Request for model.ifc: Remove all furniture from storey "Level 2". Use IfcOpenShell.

First a look at what the model holds.

```python
import ifcopenshell
import ifcopenshell.util.element

model = ifcopenshell.open("model.ifc")
print(model.schema)
storey = next(s for s in model.by_type("IfcBuildingStorey") if s.Name == "Level 2")
furniture = [e for e in ifcopenshell.util.element.get_decomposition(storey) if e.is_a("IfcFurnishingElement")]
seen = {}
for e in furniture:
    element_type = ifcopenshell.util.element.get_type(e)
    name = element_type.Name if element_type not in (None, e) else None
    seen[name] = seen.get(name, 0) + 1
for name, count in sorted(seen.items(), key=str):
    print(count, "x", name)
```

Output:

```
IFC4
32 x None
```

```python
import ifcopenshell
import ifcopenshell.api.root
import ifcopenshell.util.element

model = ifcopenshell.open("model.ifc")

storey = next(s for s in model.by_type("IfcBuildingStorey") if s.Name == "Level 2")
furniture = [e for e in ifcopenshell.util.element.get_decomposition(storey) if e.is_a("IfcFurnishingElement")]

for e in furniture:
    ifcopenshell.api.root.remove_product(model, product=e)
print(len(furniture), "removed")

model.write("model_rev.ifc")
```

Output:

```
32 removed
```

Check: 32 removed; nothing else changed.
